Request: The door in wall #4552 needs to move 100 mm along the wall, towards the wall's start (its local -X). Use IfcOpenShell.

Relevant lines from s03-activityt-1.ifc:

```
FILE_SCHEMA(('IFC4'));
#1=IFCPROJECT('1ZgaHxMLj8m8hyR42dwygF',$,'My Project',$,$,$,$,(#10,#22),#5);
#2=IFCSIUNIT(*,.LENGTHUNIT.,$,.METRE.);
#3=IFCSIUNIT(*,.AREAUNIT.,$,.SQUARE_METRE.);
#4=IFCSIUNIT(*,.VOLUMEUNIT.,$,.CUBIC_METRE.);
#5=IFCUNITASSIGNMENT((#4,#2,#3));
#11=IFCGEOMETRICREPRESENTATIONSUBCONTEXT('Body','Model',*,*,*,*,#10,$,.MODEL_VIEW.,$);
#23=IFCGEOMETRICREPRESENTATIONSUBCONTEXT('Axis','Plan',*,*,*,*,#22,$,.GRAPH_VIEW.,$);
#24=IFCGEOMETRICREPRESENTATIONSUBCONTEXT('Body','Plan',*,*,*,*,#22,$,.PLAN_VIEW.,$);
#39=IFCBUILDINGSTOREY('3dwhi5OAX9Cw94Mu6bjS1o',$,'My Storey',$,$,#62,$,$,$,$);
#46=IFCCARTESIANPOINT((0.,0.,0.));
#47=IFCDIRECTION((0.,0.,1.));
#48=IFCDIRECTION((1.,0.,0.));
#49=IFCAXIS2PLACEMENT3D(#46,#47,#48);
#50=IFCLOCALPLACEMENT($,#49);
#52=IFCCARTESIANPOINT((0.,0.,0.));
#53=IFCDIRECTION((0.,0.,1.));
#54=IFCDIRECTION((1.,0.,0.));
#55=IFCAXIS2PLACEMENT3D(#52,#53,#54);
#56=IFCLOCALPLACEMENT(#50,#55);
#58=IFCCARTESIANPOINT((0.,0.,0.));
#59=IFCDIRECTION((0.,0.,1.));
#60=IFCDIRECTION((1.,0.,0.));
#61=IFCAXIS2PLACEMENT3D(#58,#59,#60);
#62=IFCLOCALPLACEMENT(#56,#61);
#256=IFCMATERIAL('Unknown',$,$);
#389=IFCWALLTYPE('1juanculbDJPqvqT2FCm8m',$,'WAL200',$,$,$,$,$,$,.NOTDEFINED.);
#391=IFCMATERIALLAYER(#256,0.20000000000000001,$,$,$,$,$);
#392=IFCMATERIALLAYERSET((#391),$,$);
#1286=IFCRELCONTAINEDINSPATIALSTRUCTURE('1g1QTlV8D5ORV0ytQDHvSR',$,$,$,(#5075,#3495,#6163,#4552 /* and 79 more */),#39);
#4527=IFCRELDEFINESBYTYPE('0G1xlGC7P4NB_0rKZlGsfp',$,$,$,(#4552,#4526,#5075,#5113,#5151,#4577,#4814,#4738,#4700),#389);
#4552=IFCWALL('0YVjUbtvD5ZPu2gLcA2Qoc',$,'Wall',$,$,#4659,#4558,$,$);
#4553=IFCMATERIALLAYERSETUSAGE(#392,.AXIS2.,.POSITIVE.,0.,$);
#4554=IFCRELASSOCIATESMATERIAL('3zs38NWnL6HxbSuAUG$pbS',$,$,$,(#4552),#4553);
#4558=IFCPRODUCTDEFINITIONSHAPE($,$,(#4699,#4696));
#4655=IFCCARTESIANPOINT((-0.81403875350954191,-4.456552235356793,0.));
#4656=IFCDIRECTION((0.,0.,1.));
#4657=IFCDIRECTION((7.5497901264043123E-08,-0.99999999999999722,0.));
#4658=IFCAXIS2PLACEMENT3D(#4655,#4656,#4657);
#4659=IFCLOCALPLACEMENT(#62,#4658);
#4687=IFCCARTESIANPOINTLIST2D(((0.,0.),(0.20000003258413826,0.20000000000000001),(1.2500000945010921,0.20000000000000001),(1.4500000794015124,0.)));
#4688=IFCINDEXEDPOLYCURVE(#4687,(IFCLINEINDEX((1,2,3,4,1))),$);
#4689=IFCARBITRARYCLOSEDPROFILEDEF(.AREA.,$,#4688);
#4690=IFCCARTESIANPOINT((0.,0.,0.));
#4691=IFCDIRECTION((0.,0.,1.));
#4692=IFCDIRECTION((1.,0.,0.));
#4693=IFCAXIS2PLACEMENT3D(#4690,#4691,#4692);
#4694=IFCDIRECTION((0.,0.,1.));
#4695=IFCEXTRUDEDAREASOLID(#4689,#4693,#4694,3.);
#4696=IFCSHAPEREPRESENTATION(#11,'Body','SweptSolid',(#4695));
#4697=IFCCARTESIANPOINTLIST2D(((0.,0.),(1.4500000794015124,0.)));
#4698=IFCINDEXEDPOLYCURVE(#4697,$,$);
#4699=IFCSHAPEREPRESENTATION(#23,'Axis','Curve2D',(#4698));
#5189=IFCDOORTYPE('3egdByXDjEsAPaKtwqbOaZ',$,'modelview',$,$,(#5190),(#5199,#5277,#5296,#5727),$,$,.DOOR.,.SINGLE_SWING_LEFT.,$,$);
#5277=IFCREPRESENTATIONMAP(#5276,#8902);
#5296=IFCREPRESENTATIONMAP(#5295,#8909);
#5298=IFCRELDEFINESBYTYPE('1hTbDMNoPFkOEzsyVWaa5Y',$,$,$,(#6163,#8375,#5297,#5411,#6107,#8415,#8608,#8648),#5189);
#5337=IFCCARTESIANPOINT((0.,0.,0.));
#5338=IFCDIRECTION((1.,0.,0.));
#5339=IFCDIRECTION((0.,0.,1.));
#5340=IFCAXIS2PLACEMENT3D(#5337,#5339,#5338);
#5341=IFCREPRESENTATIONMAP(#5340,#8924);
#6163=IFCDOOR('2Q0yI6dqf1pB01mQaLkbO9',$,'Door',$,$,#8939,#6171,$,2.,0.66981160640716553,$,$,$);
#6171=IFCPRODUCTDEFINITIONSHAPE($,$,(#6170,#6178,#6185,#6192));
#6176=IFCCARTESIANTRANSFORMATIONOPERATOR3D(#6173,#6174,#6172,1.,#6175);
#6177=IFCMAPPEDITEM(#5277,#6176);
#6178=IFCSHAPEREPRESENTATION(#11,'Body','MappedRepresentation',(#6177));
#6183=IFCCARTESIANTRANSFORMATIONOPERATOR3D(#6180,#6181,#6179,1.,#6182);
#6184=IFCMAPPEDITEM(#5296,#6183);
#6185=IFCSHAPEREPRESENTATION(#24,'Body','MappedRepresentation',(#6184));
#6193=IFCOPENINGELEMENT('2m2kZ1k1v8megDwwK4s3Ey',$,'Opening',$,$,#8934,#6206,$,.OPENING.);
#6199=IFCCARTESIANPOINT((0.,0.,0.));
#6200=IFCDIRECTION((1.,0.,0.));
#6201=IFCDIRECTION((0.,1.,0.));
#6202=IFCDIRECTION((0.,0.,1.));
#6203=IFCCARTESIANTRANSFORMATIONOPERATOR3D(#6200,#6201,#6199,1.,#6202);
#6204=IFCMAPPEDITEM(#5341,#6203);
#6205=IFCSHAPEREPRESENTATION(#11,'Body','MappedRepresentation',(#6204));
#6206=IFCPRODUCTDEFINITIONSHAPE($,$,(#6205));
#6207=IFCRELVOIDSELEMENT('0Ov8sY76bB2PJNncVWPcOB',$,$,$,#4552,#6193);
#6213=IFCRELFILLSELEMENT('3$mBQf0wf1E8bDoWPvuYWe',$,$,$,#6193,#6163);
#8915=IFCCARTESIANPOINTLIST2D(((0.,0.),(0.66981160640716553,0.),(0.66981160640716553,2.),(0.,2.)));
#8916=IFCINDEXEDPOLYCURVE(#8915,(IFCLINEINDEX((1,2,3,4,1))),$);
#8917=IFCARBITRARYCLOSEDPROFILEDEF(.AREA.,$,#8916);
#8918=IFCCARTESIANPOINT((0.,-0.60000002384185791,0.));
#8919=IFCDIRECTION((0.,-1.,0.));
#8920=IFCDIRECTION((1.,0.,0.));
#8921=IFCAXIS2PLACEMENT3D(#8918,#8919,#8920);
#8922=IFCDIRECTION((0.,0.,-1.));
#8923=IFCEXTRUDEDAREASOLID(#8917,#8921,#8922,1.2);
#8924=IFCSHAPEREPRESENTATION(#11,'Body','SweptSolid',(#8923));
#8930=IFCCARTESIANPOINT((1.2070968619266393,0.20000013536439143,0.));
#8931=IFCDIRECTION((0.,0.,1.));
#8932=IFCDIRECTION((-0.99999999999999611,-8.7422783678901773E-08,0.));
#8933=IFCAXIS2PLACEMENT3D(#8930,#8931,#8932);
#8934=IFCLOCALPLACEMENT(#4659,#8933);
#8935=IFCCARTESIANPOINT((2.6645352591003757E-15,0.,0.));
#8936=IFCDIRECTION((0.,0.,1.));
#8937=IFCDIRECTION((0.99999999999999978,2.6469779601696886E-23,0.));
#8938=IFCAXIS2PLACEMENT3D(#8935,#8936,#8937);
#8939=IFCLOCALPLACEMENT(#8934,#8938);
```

```python
import ifcopenshell
import ifcopenshell.api.geometry
import ifcopenshell.util.placement
import ifcopenshell.util.unit

model = ifcopenshell.open("s03-activityt-1.ifc")
unit_scale = ifcopenshell.util.unit.calculate_unit_scale(model)

door = model.by_guid("2Q0yI6dqf1pB01mQaLkbO9")
opening = door.FillsVoids[0].RelatingOpeningElement
wall = opening.VoidsElements[0].RelatingBuildingElement

wall_matrix = ifcopenshell.util.placement.get_local_placement(wall.ObjectPlacement)
shift = wall_matrix[:3, 0] * -0.1 / unit_scale
before = ifcopenshell.util.placement.get_local_placement(door.ObjectPlacement)[:3, 3].copy()

# The door is placed relative to its opening, so it follows when the opening moves.
matrix = ifcopenshell.util.placement.get_local_placement(opening.ObjectPlacement)
matrix[:3, 3] += shift
ifcopenshell.api.geometry.edit_object_placement(
    model, product=opening, matrix=matrix, is_si=False, should_transform_children=True
)

after = ifcopenshell.util.placement.get_local_placement(door.ObjectPlacement)[:3, 3]
print("door moved by", (after - before).round(3) + 0.0)

model.write("s03-activityt-1-out.ifc")
```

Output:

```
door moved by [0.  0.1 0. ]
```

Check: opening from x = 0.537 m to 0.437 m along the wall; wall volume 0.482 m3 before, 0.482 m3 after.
